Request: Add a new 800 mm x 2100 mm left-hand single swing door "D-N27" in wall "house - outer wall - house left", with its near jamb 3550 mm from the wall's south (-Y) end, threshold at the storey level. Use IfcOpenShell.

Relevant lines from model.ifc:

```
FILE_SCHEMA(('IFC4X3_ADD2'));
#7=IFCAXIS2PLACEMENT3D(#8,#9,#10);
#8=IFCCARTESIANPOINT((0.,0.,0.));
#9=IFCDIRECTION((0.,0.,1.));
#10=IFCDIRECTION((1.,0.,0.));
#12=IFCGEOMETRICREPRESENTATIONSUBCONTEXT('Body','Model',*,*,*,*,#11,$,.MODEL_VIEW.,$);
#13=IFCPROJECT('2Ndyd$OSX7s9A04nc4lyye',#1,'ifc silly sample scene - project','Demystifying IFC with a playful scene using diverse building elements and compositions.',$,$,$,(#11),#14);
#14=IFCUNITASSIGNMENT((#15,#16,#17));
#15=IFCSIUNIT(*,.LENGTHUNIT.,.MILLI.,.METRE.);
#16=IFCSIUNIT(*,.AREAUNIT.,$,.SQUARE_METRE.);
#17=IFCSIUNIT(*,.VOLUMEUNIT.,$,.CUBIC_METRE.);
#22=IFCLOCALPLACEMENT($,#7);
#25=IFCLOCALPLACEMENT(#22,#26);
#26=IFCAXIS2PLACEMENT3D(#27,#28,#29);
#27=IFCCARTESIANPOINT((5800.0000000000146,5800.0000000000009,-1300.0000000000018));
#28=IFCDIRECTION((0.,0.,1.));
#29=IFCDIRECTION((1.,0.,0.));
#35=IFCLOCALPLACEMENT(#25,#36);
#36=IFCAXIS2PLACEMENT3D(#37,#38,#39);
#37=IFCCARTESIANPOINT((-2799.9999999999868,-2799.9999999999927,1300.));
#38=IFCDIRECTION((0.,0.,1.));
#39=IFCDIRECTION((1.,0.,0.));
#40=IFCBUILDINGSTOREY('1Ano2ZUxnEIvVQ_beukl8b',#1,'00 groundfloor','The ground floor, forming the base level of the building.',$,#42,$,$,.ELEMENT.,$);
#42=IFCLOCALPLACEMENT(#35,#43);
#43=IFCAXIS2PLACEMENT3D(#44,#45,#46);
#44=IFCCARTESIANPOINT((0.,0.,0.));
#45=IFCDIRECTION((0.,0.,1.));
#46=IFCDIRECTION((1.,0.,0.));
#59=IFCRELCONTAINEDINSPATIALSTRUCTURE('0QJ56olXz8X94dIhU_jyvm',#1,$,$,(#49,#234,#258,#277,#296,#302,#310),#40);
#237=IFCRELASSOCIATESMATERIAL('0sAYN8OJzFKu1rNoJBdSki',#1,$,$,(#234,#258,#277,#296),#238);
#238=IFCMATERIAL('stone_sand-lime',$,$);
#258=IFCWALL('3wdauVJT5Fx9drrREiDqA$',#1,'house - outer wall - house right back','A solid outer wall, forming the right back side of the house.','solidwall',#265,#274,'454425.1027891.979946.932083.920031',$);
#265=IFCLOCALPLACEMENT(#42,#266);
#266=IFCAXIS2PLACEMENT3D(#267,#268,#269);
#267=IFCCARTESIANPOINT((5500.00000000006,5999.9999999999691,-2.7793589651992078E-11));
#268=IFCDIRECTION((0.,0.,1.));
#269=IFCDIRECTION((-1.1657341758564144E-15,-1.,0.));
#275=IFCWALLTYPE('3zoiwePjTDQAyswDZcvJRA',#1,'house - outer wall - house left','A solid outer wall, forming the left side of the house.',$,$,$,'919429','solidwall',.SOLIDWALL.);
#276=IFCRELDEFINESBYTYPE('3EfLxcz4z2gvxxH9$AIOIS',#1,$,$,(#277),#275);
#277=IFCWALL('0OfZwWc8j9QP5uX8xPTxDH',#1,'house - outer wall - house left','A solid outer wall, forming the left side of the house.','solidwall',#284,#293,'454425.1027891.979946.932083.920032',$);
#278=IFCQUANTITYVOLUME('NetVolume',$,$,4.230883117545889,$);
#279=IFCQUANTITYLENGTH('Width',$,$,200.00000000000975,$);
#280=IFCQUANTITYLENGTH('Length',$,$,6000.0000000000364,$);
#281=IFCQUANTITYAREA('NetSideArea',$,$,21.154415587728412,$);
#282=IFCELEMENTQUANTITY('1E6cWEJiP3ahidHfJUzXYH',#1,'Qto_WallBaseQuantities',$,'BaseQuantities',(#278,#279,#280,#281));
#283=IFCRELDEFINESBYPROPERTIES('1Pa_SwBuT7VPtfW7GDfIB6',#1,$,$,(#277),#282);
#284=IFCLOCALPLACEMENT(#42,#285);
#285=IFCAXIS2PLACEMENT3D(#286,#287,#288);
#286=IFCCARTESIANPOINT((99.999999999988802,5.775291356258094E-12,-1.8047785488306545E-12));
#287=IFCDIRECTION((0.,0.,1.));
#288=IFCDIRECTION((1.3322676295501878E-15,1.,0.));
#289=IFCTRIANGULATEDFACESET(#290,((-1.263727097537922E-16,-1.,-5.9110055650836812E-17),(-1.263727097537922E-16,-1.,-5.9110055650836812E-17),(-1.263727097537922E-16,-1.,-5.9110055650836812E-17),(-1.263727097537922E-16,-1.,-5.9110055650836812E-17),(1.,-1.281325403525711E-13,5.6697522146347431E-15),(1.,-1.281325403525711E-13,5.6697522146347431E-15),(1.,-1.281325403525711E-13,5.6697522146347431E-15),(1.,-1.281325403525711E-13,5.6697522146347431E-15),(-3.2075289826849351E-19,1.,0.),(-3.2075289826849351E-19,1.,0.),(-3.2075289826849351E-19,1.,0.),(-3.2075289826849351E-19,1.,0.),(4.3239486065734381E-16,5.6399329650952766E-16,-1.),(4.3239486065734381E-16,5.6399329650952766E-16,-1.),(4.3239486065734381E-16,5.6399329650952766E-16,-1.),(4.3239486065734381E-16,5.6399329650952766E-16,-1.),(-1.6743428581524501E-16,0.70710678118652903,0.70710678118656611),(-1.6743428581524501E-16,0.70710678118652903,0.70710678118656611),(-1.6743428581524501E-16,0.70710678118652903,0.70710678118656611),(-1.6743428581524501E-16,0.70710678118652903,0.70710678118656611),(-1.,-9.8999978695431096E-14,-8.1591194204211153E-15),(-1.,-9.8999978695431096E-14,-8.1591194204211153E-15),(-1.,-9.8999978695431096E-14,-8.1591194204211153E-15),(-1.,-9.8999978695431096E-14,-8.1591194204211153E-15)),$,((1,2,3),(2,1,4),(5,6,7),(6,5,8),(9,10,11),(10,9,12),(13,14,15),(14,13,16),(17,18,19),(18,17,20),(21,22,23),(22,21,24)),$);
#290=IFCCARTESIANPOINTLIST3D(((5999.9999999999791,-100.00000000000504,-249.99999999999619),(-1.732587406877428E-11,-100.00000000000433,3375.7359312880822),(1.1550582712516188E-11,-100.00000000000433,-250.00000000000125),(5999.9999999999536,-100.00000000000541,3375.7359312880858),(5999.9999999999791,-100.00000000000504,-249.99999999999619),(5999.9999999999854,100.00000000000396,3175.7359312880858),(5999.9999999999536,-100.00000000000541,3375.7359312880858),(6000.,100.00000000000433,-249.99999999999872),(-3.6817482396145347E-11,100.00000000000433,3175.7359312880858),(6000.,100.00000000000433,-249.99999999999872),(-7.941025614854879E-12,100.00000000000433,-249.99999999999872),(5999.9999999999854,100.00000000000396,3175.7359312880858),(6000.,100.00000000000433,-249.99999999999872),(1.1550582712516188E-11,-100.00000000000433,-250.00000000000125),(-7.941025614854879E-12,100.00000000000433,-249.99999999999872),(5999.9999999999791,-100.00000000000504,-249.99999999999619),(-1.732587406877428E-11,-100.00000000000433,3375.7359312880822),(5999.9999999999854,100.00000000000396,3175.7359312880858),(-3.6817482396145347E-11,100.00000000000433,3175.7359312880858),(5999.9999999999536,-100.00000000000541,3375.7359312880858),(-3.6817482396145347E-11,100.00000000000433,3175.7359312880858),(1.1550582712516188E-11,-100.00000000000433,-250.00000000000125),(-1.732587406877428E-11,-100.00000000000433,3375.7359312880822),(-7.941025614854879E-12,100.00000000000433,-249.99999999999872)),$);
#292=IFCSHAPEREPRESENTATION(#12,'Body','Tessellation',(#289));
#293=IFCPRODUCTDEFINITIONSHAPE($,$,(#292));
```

```python
import numpy as np
import ifcopenshell
import ifcopenshell.api.feature
import ifcopenshell.api.geometry
import ifcopenshell.api.pset
import ifcopenshell.api.root
import ifcopenshell.api.spatial
import ifcopenshell.geom
import ifcopenshell.util.element
import ifcopenshell.util.placement
import ifcopenshell.util.representation
import ifcopenshell.util.shape
import ifcopenshell.util.unit

model = ifcopenshell.open("model.ifc")
unit_scale = ifcopenshell.util.unit.calculate_unit_scale(model)
area_scale = ifcopenshell.util.unit.calculate_unit_scale(model, "AREAUNIT")
volume_scale = ifcopenshell.util.unit.calculate_unit_scale(model, "VOLUMEUNIT")
settings = ifcopenshell.geom.settings()


def volume(element):
    """Net volume in cubic metres, openings subtracted."""
    shape = ifcopenshell.geom.create_shape(settings, element)
    return ifcopenshell.util.shape.get_volume(shape.geometry)


wall = model.by_guid("0OfZwWc8j9QP5uX8xPTxDH")
storey = ifcopenshell.util.element.get_container(wall, ifc_class="IfcBuildingStorey")
context = ifcopenshell.util.representation.get_context(model, "Model", "Body", "MODEL_VIEW")
before = volume(wall)

width, height, from_end, sill = 0.8, 2.1, 3.55, 0.0  # metres

# The wall runs along its own X axis, and the end named is its -X end.
wall_shape = ifcopenshell.geom.create_shape(settings, wall)
x, y, z = ifcopenshell.util.shape.get_vertices(wall_shape.geometry).T
start = x.min() + from_end
face, thickness = float(y.min()), float(y.max() - y.min())
wall_matrix = ifcopenshell.util.placement.get_local_placement(wall.ObjectPlacement)
level = ifcopenshell.util.placement.get_local_placement(storey.ObjectPlacement)[2, 3]


def in_wall(x, y):
    """Placement at x, y metres in the wall's axes, at sill height."""
    matrix = wall_matrix.copy()
    matrix[:, 3] = wall_matrix @ np.array([x / unit_scale, y / unit_scale, 0.0, 1.0])
    matrix[2, 3] = level + sill / unit_scale
    return matrix


# Opening: a box that overshoots both wall faces by 50 mm.
opening = ifcopenshell.api.root.create_entity(model, ifc_class="IfcOpeningElement", predefined_type="OPENING")
box = ifcopenshell.api.geometry.add_wall_representation(
    model, context=context, length=width, height=height, thickness=thickness + 0.1
)
ifcopenshell.api.geometry.assign_representation(model, product=opening, representation=box)
ifcopenshell.api.geometry.edit_object_placement(model, product=opening, matrix=in_wall(start, face - 0.05), is_si=False)
ifcopenshell.api.feature.add_feature(model, feature=opening, element=wall)

door = ifcopenshell.api.root.create_entity(model, ifc_class="IfcDoor", name="D-N27", predefined_type="DOOR")
door.OverallWidth, door.OverallHeight = width / unit_scale, height / unit_scale
door.OperationType = "SINGLE_SWING_LEFT"
body = ifcopenshell.api.geometry.add_door_representation(
    model,
    context=context,
    overall_width=door.OverallWidth,
    overall_height=door.OverallHeight,
    operation_type="SINGLE_SWING_LEFT",
    lining_properties={"LiningDepth": thickness / unit_scale, "ThresholdDepth": thickness / unit_scale},
)
ifcopenshell.api.geometry.assign_representation(model, product=door, representation=body)
ifcopenshell.api.spatial.assign_container(model, products=[door], relating_structure=storey)
ifcopenshell.api.feature.add_filling(model, opening=opening, element=door)

# The lining spans the wall, so the door starts at the wall face.
ifcopenshell.api.geometry.edit_object_placement(model, product=door, matrix=in_wall(start, face), is_si=False)

after = volume(wall)

# Update the wall's stored quantities.
qto = model.by_id(ifcopenshell.util.element.get_pset(wall, "Qto_WallBaseQuantities", should_inherit=False)["id"])
ifcopenshell.api.pset.edit_qto(model, qto=qto, properties={
    "NetVolume": after / volume_scale,
    "NetSideArea": after / thickness / area_scale,
})

print(f"wall volume {before:.3f} -> {after:.3f} m3")

model.write("model_edited.ifc")
```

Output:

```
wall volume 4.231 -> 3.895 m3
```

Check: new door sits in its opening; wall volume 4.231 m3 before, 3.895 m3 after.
